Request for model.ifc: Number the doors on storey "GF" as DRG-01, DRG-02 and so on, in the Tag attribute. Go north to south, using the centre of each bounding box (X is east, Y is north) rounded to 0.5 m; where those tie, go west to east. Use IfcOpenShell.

First a look at what the model holds.

```python
import ifcopenshell
import ifcopenshell.util.element
import ifcopenshell.util.placement

model = ifcopenshell.open("model.ifc")
print(model.schema)
storey = next(s for s in model.by_type("IfcBuildingStorey") if s.Name == "GF")
doors = [e for e in ifcopenshell.util.element.get_decomposition(storey) if e.is_a("IfcDoor")]
for e in sorted(doors, key=lambda e: e.id()):
    origin = ifcopenshell.util.placement.get_local_placement(e.ObjectPlacement)[:3, 3]
    print(e.id(), e.Tag, e.Name, origin.round(2) + 0.0, sep=" | ")
```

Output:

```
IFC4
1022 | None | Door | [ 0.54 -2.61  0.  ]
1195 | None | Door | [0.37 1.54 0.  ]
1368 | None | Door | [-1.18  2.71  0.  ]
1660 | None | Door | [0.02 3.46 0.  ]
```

```python
import ifcopenshell
import ifcopenshell.geom
import ifcopenshell.util.element
import ifcopenshell.util.shape

model = ifcopenshell.open("model.ifc")
settings = ifcopenshell.geom.settings()
settings.set("use-world-coords", True)


def centre(element):
    shape = ifcopenshell.geom.create_shape(settings, element)
    return ifcopenshell.util.shape.get_bbox_centroid(shape.geometry)


storey = next(s for s in model.by_type("IfcBuildingStorey") if s.Name == "GF")
doors = [e for e in ifcopenshell.util.element.get_decomposition(storey) if e.is_a("IfcDoor")]

# Insertion points can sit at a corner or the storey origin, so sort by the geometry (in metres).
centres = {e: centre(e) for e in doors}
doors.sort(key=lambda e: (-round(centres[e][1] / 0.5), centres[e][0]))

for i, e in enumerate(doors, start=1):
    number = f"DRG-{i:02d}"
    e.Tag = number
    print(e.id(), number)

model.write("model_v2.ifc")
```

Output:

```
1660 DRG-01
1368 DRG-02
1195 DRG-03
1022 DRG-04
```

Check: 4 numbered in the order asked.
